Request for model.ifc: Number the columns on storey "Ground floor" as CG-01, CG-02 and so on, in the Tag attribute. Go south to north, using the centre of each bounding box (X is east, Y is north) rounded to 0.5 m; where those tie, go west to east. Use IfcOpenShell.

First a look at what the model holds.

```python
import ifcopenshell
import ifcopenshell.util.element
import ifcopenshell.util.placement

model = ifcopenshell.open("model.ifc")
print(model.schema)
storey = next(s for s in model.by_type("IfcBuildingStorey") if s.Name == "Ground floor")
columns = [e for e in ifcopenshell.util.element.get_decomposition(storey) if e.is_a("IfcColumn")]
for e in sorted(columns, key=lambda e: e.id()):
    origin = ifcopenshell.util.placement.get_local_placement(e.ObjectPlacement)[:3, 3]
    print(e.id(), e.Tag, e.Name, origin.round(2) + 0.0, sep=" | ")
```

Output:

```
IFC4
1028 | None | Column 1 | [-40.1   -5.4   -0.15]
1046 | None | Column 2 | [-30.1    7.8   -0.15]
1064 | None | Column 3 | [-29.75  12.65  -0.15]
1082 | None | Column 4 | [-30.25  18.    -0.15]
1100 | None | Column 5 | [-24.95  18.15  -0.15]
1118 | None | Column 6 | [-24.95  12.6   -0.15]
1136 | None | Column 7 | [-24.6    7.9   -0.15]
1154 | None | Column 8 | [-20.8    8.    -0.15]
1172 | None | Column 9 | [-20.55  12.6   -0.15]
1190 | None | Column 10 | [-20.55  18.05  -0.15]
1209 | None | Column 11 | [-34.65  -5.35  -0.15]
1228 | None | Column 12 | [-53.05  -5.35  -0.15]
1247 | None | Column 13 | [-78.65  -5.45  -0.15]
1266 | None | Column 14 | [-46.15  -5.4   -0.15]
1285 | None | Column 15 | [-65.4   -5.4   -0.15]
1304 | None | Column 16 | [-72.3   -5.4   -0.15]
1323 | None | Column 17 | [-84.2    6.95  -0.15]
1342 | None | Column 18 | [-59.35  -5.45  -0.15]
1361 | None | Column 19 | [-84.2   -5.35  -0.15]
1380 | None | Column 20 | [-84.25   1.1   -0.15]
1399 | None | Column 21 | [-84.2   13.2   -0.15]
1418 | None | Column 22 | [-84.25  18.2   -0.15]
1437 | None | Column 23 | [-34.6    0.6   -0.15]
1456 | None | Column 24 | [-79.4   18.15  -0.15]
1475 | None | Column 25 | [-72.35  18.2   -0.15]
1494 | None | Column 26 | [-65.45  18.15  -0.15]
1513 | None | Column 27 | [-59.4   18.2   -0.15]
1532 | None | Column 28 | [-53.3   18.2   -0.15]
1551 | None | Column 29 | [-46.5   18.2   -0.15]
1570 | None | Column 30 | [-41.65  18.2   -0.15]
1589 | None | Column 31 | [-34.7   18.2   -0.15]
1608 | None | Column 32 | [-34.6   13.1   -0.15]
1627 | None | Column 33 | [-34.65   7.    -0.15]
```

```python
import ifcopenshell
import ifcopenshell.geom
import ifcopenshell.util.element
import ifcopenshell.util.shape

model = ifcopenshell.open("model.ifc")
settings = ifcopenshell.geom.settings()
settings.set("use-world-coords", True)


def centre(element):
    shape = ifcopenshell.geom.create_shape(settings, element)
    return ifcopenshell.util.shape.get_bbox_centroid(shape.geometry)


storey = next(s for s in model.by_type("IfcBuildingStorey") if s.Name == "Ground floor")
columns = [e for e in ifcopenshell.util.element.get_decomposition(storey) if e.is_a("IfcColumn")]

# Insertion points can sit at a corner or the storey origin, so sort by the geometry (in metres).
centres = {e: centre(e) for e in columns}
columns.sort(key=lambda e: (round(centres[e][1] / 0.5), centres[e][0]))

for i, e in enumerate(columns, start=1):
    number = f"CG-{i:02d}"
    e.Tag = number
    print(e.id(), number)

model.write("model_v2.ifc")
```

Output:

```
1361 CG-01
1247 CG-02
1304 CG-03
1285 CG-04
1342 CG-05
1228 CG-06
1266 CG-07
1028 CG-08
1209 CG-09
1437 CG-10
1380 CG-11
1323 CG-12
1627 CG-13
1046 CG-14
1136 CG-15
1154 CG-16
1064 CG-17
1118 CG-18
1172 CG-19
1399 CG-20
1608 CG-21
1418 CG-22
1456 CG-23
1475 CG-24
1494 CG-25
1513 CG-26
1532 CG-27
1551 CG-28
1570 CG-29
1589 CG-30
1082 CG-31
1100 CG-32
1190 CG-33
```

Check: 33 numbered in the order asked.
